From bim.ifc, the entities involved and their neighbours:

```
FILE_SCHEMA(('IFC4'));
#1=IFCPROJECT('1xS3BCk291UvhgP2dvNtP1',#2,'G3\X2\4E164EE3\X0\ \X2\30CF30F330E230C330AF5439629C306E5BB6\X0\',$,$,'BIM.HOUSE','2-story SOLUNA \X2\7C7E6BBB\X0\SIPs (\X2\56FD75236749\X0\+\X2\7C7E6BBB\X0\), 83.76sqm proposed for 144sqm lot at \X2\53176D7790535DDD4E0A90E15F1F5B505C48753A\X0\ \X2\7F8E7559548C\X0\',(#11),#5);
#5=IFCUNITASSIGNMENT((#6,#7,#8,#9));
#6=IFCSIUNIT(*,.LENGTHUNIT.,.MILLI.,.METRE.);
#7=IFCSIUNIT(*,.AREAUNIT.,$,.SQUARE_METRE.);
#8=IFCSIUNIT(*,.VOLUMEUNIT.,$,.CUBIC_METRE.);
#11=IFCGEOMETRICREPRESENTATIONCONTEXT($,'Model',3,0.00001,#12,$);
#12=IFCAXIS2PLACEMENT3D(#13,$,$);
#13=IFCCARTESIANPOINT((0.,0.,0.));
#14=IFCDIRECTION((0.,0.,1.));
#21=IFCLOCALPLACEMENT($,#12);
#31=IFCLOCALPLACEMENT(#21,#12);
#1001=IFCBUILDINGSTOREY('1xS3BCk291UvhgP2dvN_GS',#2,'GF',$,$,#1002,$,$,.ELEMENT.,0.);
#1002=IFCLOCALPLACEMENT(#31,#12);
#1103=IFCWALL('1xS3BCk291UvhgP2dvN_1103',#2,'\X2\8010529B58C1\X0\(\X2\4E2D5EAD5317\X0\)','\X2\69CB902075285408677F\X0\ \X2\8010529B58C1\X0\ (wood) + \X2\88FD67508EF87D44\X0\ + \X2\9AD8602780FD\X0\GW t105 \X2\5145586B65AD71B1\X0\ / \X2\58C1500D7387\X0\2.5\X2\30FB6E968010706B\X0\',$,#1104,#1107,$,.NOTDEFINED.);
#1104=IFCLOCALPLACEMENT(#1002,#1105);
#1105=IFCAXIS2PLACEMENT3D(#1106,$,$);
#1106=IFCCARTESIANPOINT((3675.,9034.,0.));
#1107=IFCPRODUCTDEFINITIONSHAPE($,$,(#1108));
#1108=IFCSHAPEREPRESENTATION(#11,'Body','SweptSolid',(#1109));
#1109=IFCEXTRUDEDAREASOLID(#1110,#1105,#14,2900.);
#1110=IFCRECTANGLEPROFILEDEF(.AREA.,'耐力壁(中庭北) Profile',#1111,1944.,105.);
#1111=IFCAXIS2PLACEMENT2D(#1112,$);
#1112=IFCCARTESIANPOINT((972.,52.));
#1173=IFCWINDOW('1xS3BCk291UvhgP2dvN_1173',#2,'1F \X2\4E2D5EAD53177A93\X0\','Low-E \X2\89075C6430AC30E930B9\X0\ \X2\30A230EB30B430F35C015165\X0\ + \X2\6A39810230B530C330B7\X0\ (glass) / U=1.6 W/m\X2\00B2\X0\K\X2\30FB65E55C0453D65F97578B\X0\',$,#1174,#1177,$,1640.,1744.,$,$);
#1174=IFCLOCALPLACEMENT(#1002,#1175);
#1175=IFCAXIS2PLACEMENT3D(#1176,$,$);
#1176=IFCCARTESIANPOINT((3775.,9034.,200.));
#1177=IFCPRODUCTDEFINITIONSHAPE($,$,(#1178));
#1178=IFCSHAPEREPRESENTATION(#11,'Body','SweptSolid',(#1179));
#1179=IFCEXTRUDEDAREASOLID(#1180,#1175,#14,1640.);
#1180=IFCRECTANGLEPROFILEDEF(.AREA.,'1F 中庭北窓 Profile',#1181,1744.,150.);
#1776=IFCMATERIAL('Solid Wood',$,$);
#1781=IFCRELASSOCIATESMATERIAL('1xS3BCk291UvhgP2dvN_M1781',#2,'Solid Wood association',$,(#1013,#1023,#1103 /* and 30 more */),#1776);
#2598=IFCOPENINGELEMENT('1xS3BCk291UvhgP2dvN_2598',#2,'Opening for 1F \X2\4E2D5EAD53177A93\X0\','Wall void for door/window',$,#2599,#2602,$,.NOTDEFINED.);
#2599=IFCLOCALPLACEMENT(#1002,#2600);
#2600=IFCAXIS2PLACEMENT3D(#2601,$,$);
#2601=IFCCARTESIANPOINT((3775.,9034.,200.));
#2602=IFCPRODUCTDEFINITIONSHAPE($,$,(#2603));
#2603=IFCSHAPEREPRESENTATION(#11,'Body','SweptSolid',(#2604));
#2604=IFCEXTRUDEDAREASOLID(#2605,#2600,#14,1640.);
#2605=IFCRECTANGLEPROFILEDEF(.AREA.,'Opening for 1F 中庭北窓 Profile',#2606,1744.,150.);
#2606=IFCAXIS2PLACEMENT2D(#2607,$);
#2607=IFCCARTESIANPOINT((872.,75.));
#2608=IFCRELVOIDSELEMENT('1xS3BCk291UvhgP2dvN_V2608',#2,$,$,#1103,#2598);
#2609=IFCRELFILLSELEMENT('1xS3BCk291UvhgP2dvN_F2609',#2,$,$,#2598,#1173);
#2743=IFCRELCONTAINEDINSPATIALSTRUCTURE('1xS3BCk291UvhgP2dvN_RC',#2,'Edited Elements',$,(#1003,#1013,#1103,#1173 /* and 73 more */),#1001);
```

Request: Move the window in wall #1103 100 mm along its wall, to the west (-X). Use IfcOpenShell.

```python
import ifcopenshell
import ifcopenshell.api.geometry
import ifcopenshell.util.placement

model = ifcopenshell.open("bim.ifc")

window = model.by_guid("1xS3BCk291UvhgP2dvN_1173")
opening = window.FillsVoids[0].RelatingOpeningElement
wall = opening.VoidsElements[0].RelatingBuildingElement

wall_matrix = ifcopenshell.util.placement.get_local_placement(wall.ObjectPlacement)
shift = wall_matrix[:3, 0] * -100.0
before = ifcopenshell.util.placement.get_local_placement(window.ObjectPlacement)[:3, 3].copy()

# The window is not placed relative to its opening, so move both.
for product in (opening, window):
    matrix = ifcopenshell.util.placement.get_local_placement(product.ObjectPlacement)
    matrix[:3, 3] += shift
    ifcopenshell.api.geometry.edit_object_placement(model, product=product, matrix=matrix, is_si=False)

after = ifcopenshell.util.placement.get_local_placement(window.ObjectPlacement)[:3, 3]
print("window moved by", (after - before).round(3) + 0.0)

model.write("bim-out.ifc")
```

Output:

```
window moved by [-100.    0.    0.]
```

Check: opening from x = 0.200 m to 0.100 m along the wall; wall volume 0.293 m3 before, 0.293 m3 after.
